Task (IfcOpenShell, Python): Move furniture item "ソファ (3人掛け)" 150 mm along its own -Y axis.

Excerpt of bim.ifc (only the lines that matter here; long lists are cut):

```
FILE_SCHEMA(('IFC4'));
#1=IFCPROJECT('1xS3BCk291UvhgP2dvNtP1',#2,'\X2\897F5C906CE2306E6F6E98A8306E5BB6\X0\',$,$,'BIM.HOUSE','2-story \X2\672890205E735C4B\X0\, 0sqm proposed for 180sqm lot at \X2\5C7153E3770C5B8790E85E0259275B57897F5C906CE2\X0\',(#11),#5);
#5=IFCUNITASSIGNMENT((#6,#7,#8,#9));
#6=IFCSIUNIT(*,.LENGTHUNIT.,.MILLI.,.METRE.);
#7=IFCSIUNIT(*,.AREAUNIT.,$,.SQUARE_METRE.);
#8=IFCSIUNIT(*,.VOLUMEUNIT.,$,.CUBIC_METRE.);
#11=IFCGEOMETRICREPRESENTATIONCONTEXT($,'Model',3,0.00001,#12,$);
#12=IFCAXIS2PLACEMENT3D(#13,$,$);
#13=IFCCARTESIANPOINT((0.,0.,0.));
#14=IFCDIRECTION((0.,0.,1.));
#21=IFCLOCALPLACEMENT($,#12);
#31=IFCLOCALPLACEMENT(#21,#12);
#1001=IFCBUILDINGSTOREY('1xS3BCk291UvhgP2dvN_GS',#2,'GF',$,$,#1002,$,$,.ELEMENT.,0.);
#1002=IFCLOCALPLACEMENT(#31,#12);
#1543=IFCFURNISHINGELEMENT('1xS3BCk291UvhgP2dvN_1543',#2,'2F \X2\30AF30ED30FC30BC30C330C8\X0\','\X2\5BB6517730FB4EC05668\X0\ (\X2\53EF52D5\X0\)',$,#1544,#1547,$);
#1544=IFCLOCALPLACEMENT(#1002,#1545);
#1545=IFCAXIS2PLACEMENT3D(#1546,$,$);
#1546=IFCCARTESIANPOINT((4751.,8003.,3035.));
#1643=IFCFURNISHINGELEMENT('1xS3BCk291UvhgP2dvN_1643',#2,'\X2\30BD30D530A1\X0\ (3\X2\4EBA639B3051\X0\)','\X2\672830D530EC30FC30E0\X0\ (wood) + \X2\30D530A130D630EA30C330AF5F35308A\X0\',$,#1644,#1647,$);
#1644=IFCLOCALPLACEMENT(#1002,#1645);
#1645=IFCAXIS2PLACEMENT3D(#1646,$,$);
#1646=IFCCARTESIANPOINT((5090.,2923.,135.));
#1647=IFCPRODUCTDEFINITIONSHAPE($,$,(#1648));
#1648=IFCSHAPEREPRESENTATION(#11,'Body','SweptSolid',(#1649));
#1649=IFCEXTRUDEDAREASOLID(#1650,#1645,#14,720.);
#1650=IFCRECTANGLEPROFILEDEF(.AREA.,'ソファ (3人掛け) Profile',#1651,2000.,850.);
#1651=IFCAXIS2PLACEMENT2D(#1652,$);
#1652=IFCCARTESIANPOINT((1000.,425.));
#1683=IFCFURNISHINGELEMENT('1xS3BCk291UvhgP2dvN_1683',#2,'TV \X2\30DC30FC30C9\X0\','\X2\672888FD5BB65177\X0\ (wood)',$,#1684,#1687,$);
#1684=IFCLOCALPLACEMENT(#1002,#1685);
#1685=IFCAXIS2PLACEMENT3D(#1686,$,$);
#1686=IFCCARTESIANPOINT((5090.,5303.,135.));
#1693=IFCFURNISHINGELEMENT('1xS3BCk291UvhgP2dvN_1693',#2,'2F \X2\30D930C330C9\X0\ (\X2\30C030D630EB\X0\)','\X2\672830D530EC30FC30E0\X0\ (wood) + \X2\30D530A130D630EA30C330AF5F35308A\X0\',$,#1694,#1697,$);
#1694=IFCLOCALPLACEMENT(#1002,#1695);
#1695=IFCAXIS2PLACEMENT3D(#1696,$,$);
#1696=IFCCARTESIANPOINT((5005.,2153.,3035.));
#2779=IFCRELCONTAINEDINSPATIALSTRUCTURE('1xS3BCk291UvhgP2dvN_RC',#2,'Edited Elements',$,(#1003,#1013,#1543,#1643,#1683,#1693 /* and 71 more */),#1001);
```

```python
import ifcopenshell
import ifcopenshell.api.geometry
import ifcopenshell.util.placement

model = ifcopenshell.open("bim.ifc")

item = model.by_guid("1xS3BCk291UvhgP2dvN_1643")
matrix = ifcopenshell.util.placement.get_local_placement(item.ObjectPlacement)
matrix[:3, 3] -= matrix[:3, 1] * 150.0
ifcopenshell.api.geometry.edit_object_placement(model, product=item, matrix=matrix, is_si=False)

print(ifcopenshell.util.placement.get_local_placement(item.ObjectPlacement).round(3) + 0.0)

model.write("bim_updated.ifc")
```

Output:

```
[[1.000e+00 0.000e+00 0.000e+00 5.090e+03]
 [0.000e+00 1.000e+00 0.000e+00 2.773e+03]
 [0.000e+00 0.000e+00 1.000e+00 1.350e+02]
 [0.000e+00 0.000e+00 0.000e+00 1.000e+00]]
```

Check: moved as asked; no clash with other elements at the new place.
